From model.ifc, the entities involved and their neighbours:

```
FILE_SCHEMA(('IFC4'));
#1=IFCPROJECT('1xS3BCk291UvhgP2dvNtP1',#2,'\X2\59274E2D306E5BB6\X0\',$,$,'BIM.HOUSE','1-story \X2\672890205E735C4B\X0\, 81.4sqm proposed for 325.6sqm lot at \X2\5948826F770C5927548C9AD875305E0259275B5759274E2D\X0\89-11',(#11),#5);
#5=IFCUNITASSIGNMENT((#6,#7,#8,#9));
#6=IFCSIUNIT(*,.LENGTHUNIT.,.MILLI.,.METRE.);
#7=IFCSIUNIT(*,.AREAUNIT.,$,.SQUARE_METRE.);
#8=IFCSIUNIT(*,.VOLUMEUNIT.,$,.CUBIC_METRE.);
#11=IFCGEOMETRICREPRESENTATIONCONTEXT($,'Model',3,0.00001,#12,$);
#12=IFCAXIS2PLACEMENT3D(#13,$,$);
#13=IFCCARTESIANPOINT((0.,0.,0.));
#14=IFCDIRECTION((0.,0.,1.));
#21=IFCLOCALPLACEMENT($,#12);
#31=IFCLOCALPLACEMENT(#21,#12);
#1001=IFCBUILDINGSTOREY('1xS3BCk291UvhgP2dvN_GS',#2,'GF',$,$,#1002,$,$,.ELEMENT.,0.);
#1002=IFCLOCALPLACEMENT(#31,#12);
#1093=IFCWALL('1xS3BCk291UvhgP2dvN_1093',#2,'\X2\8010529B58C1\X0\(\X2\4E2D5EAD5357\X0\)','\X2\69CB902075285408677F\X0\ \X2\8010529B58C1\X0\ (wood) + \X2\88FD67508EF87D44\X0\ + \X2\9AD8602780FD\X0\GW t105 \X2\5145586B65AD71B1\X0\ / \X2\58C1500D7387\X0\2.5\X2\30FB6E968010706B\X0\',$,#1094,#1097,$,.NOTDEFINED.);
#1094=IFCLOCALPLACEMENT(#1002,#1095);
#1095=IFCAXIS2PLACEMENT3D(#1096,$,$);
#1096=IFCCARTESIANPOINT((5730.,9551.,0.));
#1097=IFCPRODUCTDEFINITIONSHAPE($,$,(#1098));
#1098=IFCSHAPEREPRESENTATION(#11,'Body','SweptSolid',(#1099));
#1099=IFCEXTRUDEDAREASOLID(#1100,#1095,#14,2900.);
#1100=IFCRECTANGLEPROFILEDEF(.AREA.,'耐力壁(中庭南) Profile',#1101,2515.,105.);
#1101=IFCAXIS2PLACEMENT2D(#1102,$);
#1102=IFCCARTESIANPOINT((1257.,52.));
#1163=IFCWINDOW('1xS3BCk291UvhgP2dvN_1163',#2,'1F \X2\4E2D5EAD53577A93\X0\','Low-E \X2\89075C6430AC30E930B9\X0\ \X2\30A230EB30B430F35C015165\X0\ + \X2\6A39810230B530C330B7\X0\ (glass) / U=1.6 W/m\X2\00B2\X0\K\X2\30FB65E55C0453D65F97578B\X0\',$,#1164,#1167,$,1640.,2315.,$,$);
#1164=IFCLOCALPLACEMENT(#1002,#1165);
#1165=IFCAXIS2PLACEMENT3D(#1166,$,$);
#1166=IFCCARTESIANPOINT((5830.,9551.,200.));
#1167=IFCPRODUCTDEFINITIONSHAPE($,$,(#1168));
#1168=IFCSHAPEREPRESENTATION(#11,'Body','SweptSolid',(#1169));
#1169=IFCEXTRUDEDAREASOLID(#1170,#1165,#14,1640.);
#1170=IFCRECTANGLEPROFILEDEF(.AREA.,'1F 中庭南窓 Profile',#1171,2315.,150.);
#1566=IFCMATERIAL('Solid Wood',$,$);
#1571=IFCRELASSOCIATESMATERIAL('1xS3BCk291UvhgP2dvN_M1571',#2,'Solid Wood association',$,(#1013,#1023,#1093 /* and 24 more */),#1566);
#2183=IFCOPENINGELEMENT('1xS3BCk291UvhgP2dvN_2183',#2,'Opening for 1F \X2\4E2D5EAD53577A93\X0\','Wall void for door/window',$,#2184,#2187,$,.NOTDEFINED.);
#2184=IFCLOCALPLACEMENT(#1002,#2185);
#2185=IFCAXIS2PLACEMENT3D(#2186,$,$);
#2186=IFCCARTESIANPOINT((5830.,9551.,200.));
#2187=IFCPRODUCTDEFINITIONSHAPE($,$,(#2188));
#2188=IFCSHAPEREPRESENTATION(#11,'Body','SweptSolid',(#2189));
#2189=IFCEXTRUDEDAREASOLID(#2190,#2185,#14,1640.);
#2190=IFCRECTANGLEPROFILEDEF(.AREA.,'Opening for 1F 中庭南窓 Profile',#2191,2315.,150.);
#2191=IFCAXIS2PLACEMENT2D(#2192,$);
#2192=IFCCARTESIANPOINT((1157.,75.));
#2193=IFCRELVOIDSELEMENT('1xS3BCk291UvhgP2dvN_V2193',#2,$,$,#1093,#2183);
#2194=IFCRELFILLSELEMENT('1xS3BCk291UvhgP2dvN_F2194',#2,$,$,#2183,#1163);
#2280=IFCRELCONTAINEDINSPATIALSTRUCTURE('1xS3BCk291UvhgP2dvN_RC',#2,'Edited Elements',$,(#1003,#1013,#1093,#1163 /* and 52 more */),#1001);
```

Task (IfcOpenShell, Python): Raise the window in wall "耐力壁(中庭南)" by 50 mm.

```python
import numpy as np
import ifcopenshell
import ifcopenshell.api.geometry
import ifcopenshell.util.placement
import ifcopenshell.util.unit

model = ifcopenshell.open("model.ifc")
unit_scale = ifcopenshell.util.unit.calculate_unit_scale(model)

window = model.by_guid("1xS3BCk291UvhgP2dvN_1163")
opening = window.FillsVoids[0].RelatingOpeningElement
dz = 50.0

shift = np.array([0.0, 0.0, dz])
# The window is not placed relative to its opening, so move both.
for product in (opening, window):
    matrix = ifcopenshell.util.placement.get_local_placement(product.ObjectPlacement)
    matrix[:3, 3] += shift
    ifcopenshell.api.geometry.edit_object_placement(model, product=product, matrix=matrix, is_si=False)

print(f"moved by {dz * unit_scale:+.3f} m")

model.write("model_rev.ifc")
```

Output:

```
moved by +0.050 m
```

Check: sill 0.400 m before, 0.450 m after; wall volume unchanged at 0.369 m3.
